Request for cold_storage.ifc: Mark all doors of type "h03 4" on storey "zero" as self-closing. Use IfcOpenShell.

First a look at what the model holds.

```python
import ifcopenshell
import ifcopenshell.util.element

model = ifcopenshell.open("cold_storage.ifc")
print(model.schema)
storey = next(s for s in model.by_type("IfcBuildingStorey") if s.Name == "zero")
doors = [e for e in ifcopenshell.util.element.get_decomposition(storey) if e.is_a("IfcDoor")]
seen = {}
for e in doors:
    element_type = ifcopenshell.util.element.get_type(e)
    key = (element_type.Name if element_type != e and element_type else None, ifcopenshell.util.element.get_pset(e, "Pset_DoorCommon", "SelfClosing"))
    seen[key] = seen.get(key, 0) + 1
for (name, value), count in sorted(seen.items(), key=str):
    print(count, "x", name, "|", value)
```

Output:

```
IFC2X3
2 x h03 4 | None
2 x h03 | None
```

```python
import ifcopenshell
import ifcopenshell.api.pset
import ifcopenshell.util.element

model = ifcopenshell.open("cold_storage.ifc")

storey = next(s for s in model.by_type("IfcBuildingStorey") if s.Name == "zero")
doors = [e for e in ifcopenshell.util.element.get_decomposition(storey) if e.is_a("IfcDoor")]

count = 0
for e in doors:
    element_type = ifcopenshell.util.element.get_type(e)
    if element_type in (None, e) or element_type.Name != "h03 4":
        continue
    # add_pset returns the element's existing set when there is one.
    pset = ifcopenshell.api.pset.add_pset(model, product=e, name="Pset_DoorCommon")
    ifcopenshell.api.pset.edit_pset(model, pset=pset, properties={"SelfClosing": True})
    count += 1

print(count, "doors updated")

model.write("cold_storage_edited.ifc")
```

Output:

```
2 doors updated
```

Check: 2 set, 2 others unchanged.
